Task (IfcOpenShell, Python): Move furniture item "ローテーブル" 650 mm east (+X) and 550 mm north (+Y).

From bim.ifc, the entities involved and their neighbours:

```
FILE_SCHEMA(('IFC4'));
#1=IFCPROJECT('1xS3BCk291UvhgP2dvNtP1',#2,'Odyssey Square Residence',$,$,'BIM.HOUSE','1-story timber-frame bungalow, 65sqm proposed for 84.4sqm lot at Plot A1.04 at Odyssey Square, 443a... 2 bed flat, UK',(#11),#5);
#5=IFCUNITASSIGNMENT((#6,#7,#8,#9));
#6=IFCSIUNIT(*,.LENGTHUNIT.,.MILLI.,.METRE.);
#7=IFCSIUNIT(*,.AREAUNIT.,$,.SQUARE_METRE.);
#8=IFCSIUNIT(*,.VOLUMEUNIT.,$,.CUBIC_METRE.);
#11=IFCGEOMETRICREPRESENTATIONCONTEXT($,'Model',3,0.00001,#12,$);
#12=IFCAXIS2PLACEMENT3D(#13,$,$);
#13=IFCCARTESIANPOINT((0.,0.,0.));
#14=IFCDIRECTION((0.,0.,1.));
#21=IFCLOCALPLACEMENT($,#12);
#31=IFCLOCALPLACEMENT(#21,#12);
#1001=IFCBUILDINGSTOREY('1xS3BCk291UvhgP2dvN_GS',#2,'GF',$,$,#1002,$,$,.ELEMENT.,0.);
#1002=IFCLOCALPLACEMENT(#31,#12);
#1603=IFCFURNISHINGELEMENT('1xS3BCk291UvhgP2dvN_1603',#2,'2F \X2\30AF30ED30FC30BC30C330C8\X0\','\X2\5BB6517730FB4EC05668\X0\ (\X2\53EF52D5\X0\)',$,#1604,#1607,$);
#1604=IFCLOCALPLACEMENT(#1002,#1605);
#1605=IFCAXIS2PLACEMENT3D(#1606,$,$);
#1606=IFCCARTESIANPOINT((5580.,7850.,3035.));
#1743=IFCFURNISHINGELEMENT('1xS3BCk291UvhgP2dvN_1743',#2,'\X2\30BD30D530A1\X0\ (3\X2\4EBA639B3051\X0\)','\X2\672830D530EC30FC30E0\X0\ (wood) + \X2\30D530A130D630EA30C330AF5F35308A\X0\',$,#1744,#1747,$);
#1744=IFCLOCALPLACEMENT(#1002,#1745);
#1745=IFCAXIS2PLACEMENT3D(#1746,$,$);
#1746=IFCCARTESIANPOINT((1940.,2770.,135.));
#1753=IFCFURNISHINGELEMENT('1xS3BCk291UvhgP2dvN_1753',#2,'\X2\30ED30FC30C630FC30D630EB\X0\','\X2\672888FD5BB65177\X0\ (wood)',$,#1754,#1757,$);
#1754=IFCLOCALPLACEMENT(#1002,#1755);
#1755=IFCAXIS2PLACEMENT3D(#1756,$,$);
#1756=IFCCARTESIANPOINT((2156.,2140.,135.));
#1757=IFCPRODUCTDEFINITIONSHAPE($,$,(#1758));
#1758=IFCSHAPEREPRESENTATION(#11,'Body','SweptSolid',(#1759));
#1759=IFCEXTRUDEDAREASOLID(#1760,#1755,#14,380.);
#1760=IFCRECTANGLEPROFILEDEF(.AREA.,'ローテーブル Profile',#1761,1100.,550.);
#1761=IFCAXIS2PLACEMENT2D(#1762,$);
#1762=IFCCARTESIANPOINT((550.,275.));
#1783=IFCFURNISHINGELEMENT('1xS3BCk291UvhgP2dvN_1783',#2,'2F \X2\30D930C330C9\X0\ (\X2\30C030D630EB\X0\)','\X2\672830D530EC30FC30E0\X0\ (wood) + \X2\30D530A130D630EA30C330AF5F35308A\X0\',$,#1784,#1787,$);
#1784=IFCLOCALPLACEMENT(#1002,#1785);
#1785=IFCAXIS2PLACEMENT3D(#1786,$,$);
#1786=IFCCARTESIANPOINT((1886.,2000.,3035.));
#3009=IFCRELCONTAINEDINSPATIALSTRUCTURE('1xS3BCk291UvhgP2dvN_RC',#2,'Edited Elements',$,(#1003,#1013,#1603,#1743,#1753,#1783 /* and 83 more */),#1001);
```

```python
import ifcopenshell
import ifcopenshell.api.geometry
import ifcopenshell.util.placement
import ifcopenshell.util.unit

model = ifcopenshell.open("bim.ifc")
unit_scale = ifcopenshell.util.unit.calculate_unit_scale(model)

item = model.by_guid("1xS3BCk291UvhgP2dvN_1753")
matrix = ifcopenshell.util.placement.get_local_placement(item.ObjectPlacement)
matrix[0, 3] += 0.65 / unit_scale
matrix[1, 3] += 0.55 / unit_scale
ifcopenshell.api.geometry.edit_object_placement(model, product=item, matrix=matrix, is_si=False)

print(ifcopenshell.util.placement.get_local_placement(item.ObjectPlacement).round(3) + 0.0)

model.write("bim_edited.ifc")
```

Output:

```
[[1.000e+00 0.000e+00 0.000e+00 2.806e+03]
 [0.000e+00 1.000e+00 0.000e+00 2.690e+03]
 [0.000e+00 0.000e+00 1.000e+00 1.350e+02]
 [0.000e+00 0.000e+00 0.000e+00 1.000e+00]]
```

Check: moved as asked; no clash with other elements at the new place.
